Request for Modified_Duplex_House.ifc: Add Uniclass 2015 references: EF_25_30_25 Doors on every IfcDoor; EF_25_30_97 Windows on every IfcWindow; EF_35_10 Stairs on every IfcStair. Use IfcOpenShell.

First a look at what the model holds.

```python
import ifcopenshell

model = ifcopenshell.open("Modified_Duplex_House.ifc")
print(model.schema)
print("classifications:", [c.Name for c in model.by_type("IfcClassification")])
for ifc_class in ("IfcDoor", "IfcRoof", "IfcStair", "IfcWall", "IfcWindow"):
    print(ifc_class, len(model.by_type(ifc_class)))
```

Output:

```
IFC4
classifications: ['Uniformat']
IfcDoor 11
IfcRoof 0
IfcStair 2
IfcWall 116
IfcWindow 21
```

```python
import ifcopenshell
import ifcopenshell.api.classification

model = ifcopenshell.open("Modified_Duplex_House.ifc")

system = ifcopenshell.api.classification.add_classification(model, classification="Uniclass 2015")

codes = {
    "IfcDoor": ("EF_25_30_25", "Doors"),
    "IfcWindow": ("EF_25_30_97", "Windows"),
    "IfcStair": ("EF_35_10", "Stairs"),
}
for ifc_class, (code, name) in codes.items():
    products = model.by_type(ifc_class)
    ifcopenshell.api.classification.add_reference(
        model, products=products, classification=system, identification=code, name=name
    )
    print(code, len(products))

model.write("Modified_Duplex_House_edited.ifc")
```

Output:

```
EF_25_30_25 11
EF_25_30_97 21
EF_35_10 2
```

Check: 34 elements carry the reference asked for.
